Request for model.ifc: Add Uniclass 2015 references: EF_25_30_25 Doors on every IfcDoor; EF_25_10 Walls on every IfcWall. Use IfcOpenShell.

First a look at what the model holds.

```python
import ifcopenshell

model = ifcopenshell.open("model.ifc")
print(model.schema)
print("classifications:", [c.Name for c in model.by_type("IfcClassification")])
for ifc_class in ("IfcDoor", "IfcRoof", "IfcStair", "IfcWall", "IfcWindow"):
    print(ifc_class, len(model.by_type(ifc_class)))
```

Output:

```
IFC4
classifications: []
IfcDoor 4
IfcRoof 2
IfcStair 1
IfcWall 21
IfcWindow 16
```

```python
import ifcopenshell
import ifcopenshell.api.classification

model = ifcopenshell.open("model.ifc")

system = ifcopenshell.api.classification.add_classification(model, classification="Uniclass 2015")

codes = {
    "IfcDoor": ("EF_25_30_25", "Doors"),
    "IfcWall": ("EF_25_10", "Walls"),
}
for ifc_class, (code, name) in codes.items():
    products = model.by_type(ifc_class)
    ifcopenshell.api.classification.add_reference(
        model, products=products, classification=system, identification=code, name=name
    )
    print(code, len(products))

model.write("model_v2.ifc")
```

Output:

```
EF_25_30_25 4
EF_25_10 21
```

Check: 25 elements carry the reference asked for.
